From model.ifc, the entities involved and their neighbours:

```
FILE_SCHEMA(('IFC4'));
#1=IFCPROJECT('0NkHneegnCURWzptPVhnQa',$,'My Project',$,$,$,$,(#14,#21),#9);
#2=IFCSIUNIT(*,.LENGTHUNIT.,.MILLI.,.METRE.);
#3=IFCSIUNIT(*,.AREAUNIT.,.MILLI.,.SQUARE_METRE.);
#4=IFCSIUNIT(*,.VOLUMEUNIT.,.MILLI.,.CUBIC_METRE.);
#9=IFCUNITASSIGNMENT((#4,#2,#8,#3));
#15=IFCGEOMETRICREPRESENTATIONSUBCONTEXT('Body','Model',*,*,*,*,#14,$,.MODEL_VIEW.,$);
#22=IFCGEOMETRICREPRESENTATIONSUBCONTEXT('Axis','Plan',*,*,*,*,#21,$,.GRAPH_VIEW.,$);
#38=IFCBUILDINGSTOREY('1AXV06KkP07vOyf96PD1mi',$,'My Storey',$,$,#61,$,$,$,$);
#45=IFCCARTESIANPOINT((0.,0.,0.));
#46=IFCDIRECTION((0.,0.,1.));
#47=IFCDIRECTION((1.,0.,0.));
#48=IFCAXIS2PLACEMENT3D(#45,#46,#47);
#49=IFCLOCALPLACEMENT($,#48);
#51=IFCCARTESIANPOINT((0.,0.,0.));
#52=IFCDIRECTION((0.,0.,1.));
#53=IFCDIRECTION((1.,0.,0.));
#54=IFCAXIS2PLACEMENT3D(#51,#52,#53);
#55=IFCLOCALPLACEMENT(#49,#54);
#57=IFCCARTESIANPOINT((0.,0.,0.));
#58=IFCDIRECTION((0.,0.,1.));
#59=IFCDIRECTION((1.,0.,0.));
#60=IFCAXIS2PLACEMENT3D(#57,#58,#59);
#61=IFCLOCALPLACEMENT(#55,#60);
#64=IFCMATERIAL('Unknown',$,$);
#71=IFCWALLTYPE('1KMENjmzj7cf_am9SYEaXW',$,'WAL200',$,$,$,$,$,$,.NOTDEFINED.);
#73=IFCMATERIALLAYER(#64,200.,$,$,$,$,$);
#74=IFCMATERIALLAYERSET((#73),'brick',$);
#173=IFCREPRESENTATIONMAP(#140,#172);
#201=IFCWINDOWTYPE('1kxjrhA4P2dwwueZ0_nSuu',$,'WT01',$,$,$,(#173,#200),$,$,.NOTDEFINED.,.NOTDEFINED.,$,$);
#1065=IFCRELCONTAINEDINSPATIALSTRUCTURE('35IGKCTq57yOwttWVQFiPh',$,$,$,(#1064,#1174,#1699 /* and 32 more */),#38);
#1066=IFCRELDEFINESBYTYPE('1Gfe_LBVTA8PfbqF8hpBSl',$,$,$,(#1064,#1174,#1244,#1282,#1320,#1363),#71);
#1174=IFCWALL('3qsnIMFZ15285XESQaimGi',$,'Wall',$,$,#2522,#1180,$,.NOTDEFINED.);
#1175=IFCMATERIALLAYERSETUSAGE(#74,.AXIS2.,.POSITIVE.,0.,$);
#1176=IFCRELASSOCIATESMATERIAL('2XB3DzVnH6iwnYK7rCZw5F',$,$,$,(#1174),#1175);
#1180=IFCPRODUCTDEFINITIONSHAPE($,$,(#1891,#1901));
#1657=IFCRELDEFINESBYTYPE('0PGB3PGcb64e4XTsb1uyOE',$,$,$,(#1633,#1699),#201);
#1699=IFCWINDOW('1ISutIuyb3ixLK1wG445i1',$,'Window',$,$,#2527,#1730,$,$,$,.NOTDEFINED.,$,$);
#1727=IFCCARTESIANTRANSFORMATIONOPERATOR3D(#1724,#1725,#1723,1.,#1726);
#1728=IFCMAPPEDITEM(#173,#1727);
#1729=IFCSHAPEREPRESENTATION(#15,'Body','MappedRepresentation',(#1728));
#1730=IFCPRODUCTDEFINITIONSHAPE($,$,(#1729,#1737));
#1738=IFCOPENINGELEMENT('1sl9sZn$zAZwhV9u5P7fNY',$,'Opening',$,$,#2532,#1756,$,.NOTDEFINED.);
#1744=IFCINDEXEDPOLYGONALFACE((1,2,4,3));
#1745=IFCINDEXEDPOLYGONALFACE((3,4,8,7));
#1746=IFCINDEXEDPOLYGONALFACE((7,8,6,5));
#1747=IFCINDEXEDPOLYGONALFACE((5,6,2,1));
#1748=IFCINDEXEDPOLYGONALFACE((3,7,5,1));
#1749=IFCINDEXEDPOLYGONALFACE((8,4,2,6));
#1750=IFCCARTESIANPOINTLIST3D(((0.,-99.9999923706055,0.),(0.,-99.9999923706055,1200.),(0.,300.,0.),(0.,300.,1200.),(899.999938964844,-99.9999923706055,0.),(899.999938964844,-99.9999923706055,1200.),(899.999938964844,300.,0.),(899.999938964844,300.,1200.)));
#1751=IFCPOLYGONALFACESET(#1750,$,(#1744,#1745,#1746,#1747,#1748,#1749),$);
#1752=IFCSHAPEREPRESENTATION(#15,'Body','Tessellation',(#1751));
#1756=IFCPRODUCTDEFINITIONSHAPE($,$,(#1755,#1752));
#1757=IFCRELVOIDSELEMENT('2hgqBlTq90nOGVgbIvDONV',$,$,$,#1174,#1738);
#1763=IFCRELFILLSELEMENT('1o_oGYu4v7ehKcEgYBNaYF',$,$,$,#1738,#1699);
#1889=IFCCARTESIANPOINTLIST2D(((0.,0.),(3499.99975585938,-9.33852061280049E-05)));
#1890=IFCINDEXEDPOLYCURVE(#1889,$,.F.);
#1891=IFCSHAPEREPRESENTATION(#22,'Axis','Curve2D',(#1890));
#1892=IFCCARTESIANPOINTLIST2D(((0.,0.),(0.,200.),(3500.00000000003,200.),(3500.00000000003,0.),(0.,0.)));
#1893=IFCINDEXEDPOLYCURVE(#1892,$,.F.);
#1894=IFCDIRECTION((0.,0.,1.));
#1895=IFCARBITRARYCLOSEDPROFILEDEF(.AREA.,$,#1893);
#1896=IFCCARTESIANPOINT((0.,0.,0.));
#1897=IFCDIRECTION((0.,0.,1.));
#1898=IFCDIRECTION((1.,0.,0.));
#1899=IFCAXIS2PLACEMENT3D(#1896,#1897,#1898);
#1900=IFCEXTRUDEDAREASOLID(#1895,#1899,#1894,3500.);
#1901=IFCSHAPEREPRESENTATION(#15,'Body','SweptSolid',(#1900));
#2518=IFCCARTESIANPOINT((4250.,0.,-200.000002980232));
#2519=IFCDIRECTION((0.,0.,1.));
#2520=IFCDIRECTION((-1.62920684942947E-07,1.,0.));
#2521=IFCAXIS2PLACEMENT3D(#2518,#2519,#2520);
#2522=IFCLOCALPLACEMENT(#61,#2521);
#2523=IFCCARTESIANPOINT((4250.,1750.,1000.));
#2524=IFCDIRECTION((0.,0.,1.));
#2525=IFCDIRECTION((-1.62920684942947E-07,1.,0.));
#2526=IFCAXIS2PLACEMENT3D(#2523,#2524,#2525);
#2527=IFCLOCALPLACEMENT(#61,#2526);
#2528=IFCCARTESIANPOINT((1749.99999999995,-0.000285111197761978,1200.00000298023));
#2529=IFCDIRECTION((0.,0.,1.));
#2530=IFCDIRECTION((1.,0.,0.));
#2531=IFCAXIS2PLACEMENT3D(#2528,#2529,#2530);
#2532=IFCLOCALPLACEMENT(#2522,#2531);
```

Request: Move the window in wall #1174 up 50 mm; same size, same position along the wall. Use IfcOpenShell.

```python
import numpy as np
import ifcopenshell
import ifcopenshell.api.geometry
import ifcopenshell.util.placement
import ifcopenshell.util.unit

model = ifcopenshell.open("model.ifc")
unit_scale = ifcopenshell.util.unit.calculate_unit_scale(model)

window = model.by_guid("1ISutIuyb3ixLK1wG445i1")
opening = window.FillsVoids[0].RelatingOpeningElement
dz = 0.05 / unit_scale

shift = np.array([0.0, 0.0, dz])
# The window is not placed relative to its opening, so move both.
for product in (opening, window):
    matrix = ifcopenshell.util.placement.get_local_placement(product.ObjectPlacement)
    matrix[:3, 3] += shift
    ifcopenshell.api.geometry.edit_object_placement(model, product=product, matrix=matrix, is_si=False)

print(f"moved by {dz * unit_scale:+.3f} m")

model.write("model_v2.ifc")
```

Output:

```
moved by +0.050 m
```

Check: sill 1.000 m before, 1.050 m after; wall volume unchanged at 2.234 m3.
